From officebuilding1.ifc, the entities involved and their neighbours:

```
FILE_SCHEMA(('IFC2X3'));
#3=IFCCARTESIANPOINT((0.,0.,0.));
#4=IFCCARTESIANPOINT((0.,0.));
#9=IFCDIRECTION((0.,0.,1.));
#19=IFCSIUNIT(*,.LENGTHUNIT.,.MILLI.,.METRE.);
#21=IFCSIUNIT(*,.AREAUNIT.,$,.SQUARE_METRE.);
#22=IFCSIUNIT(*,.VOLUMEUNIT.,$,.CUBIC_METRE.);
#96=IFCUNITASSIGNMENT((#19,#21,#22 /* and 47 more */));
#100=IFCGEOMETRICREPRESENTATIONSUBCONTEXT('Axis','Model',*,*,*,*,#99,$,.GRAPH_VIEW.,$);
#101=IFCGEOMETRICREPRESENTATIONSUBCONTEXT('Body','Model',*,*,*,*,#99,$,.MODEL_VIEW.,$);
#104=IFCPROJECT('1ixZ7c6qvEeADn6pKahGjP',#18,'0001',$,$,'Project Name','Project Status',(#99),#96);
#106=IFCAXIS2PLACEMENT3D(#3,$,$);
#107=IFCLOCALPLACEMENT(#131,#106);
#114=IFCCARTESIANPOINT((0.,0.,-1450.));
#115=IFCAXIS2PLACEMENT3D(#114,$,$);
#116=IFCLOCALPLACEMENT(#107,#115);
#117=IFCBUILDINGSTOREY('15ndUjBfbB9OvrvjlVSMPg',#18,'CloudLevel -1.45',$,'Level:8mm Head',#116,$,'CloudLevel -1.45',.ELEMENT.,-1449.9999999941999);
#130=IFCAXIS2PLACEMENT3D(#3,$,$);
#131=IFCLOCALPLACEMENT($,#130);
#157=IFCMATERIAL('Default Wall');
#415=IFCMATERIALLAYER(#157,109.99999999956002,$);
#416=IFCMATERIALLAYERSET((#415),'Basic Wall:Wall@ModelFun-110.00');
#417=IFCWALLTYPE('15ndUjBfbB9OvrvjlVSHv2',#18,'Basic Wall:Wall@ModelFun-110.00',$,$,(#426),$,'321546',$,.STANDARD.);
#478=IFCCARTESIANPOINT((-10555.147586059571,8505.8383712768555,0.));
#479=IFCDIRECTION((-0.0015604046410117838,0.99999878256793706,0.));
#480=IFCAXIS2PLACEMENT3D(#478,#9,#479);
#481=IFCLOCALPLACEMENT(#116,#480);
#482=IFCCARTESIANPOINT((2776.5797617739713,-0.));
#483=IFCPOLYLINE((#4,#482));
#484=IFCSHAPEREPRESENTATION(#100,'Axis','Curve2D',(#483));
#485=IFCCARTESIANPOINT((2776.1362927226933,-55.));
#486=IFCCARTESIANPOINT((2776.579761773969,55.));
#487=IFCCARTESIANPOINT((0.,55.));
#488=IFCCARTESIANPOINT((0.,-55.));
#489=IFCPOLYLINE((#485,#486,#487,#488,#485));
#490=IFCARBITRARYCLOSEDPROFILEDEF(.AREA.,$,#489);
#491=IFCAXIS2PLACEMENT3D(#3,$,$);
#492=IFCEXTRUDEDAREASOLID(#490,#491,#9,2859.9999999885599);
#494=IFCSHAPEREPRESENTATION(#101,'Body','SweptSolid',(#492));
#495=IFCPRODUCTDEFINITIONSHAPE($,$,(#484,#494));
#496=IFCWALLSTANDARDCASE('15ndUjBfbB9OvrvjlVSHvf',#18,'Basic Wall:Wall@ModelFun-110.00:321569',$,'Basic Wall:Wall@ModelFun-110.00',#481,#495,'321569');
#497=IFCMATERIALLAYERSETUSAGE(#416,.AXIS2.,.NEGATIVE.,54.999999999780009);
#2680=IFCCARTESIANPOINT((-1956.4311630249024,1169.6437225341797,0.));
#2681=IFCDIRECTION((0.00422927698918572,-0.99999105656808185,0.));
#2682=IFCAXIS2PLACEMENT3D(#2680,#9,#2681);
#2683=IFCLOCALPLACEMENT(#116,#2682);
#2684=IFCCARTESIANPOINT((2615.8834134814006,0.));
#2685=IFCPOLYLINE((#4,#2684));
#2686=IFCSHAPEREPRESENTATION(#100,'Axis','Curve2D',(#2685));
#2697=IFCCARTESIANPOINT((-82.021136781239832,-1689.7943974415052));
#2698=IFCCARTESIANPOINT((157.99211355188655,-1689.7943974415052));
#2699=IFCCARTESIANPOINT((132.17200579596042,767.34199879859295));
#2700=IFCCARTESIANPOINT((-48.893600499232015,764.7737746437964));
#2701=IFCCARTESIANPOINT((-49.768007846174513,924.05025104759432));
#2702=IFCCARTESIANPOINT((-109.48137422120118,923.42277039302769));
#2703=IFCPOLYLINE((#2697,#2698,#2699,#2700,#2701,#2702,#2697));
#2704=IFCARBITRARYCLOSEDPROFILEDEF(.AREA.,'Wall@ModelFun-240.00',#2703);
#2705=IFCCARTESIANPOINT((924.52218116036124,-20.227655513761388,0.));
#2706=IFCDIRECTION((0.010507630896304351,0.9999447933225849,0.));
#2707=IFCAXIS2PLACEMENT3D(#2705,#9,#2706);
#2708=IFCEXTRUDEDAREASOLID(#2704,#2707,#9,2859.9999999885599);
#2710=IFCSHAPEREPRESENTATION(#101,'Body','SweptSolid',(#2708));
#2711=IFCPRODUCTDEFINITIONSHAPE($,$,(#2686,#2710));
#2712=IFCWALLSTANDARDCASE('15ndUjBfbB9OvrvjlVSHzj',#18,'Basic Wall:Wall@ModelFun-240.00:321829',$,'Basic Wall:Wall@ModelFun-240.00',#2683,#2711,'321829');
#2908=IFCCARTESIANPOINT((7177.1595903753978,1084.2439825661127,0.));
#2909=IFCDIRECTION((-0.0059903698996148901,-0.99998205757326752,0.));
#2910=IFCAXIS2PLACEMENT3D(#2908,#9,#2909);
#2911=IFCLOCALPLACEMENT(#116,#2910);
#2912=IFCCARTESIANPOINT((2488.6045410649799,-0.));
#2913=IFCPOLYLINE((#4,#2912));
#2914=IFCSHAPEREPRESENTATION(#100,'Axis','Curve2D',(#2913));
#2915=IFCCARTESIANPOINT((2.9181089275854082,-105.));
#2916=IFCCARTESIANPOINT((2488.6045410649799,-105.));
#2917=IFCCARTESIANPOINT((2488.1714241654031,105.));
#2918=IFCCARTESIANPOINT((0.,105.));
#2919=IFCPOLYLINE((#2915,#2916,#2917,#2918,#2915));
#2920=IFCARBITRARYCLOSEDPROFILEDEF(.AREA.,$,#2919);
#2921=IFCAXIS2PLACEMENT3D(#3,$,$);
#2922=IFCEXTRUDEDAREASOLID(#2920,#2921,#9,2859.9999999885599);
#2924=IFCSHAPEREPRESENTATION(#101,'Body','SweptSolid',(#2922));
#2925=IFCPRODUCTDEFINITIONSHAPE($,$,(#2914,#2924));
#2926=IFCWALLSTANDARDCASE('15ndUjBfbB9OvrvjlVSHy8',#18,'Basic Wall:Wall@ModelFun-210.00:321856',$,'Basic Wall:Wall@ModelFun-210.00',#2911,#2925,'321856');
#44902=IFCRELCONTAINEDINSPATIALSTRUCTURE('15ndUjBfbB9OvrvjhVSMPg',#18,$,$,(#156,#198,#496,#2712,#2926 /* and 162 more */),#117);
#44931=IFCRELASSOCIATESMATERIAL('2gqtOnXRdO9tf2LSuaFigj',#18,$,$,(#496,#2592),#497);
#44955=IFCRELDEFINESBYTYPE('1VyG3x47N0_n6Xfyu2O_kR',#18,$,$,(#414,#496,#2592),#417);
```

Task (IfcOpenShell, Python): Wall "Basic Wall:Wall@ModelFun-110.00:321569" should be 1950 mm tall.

```python
import ifcopenshell
import ifcopenshell.geom
import ifcopenshell.util.representation
import ifcopenshell.util.shape

model = ifcopenshell.open("officebuilding1.ifc")
settings = ifcopenshell.geom.settings()


def volume(element):
    """Net volume in cubic metres, openings subtracted."""
    shape = ifcopenshell.geom.create_shape(settings, element)
    return ifcopenshell.util.shape.get_volume(shape.geometry)


wall = model.by_guid("15ndUjBfbB9OvrvjlVSHvf")
before = volume(wall)

body = ifcopenshell.util.representation.get_representation(wall, "Model", "Body")
solid = body.Items[0]
old_height = solid.Depth
solid.Depth = 1950.0
after = volume(wall)

print(f"height {old_height:g} -> {solid.Depth:g}, volume {before:.3f} -> {after:.3f} m3")

model.write("officebuilding1_v2.ifc")
```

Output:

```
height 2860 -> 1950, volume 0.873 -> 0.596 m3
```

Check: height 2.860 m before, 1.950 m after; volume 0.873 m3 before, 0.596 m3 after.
